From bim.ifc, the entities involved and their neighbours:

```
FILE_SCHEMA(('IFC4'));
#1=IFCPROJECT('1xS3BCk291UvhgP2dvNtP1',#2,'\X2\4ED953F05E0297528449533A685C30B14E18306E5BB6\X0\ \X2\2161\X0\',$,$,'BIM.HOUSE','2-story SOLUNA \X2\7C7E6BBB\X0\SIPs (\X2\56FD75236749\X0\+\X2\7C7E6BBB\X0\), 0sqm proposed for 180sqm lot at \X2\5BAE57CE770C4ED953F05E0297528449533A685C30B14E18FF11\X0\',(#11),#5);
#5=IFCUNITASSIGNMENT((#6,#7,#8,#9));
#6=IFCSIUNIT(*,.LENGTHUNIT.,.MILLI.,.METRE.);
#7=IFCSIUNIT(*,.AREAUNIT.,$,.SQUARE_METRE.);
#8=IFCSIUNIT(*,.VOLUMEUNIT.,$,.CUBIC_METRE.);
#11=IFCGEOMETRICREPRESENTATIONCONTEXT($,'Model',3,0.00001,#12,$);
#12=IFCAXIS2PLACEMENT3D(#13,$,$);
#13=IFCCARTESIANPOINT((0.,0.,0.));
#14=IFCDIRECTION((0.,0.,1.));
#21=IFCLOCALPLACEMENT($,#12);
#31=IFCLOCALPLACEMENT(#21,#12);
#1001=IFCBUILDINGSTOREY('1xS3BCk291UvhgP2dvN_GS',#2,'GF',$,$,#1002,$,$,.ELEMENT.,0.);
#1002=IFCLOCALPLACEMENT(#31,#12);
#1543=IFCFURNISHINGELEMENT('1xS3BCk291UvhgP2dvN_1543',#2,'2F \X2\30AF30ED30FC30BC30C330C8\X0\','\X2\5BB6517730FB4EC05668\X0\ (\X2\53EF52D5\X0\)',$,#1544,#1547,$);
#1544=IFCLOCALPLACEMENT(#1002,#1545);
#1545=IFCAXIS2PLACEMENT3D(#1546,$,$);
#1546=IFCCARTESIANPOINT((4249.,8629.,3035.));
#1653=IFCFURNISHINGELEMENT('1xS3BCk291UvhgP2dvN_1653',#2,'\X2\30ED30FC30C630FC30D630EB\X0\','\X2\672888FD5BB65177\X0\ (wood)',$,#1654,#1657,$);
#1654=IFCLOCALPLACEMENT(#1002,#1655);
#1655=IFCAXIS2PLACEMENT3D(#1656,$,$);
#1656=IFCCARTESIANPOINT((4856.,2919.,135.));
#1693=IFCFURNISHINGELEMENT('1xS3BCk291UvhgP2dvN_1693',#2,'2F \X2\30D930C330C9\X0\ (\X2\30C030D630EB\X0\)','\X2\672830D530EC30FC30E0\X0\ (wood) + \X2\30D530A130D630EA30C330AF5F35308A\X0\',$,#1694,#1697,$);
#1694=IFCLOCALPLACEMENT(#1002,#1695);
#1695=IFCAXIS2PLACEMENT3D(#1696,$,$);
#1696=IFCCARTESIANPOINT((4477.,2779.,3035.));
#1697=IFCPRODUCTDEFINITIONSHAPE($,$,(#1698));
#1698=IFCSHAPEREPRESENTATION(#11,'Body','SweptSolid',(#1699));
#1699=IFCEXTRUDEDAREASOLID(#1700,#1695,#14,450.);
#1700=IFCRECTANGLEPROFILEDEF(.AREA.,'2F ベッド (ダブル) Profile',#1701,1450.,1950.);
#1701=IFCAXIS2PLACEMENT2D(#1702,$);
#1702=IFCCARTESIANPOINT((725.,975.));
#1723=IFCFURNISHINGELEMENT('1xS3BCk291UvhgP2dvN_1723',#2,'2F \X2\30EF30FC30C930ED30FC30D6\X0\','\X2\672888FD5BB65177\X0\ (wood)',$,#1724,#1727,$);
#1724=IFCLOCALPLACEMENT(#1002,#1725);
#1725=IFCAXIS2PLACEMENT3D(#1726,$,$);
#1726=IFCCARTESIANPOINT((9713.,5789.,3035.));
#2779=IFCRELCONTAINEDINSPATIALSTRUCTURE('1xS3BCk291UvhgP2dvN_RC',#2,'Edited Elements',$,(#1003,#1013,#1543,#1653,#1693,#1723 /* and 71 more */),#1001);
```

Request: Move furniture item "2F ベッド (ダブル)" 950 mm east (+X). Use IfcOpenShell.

```python
import ifcopenshell
import ifcopenshell.api.geometry
import ifcopenshell.util.placement
import ifcopenshell.util.unit

model = ifcopenshell.open("bim.ifc")
unit_scale = ifcopenshell.util.unit.calculate_unit_scale(model)

item = model.by_guid("1xS3BCk291UvhgP2dvN_1693")
matrix = ifcopenshell.util.placement.get_local_placement(item.ObjectPlacement)
matrix[0, 3] += 0.95 / unit_scale
ifcopenshell.api.geometry.edit_object_placement(model, product=item, matrix=matrix, is_si=False)

print(ifcopenshell.util.placement.get_local_placement(item.ObjectPlacement).round(3) + 0.0)

model.write("bim_edited.ifc")
```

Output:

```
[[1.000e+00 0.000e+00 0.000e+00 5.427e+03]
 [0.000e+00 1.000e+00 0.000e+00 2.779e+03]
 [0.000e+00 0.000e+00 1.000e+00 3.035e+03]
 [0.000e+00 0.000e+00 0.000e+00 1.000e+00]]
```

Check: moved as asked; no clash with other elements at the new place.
